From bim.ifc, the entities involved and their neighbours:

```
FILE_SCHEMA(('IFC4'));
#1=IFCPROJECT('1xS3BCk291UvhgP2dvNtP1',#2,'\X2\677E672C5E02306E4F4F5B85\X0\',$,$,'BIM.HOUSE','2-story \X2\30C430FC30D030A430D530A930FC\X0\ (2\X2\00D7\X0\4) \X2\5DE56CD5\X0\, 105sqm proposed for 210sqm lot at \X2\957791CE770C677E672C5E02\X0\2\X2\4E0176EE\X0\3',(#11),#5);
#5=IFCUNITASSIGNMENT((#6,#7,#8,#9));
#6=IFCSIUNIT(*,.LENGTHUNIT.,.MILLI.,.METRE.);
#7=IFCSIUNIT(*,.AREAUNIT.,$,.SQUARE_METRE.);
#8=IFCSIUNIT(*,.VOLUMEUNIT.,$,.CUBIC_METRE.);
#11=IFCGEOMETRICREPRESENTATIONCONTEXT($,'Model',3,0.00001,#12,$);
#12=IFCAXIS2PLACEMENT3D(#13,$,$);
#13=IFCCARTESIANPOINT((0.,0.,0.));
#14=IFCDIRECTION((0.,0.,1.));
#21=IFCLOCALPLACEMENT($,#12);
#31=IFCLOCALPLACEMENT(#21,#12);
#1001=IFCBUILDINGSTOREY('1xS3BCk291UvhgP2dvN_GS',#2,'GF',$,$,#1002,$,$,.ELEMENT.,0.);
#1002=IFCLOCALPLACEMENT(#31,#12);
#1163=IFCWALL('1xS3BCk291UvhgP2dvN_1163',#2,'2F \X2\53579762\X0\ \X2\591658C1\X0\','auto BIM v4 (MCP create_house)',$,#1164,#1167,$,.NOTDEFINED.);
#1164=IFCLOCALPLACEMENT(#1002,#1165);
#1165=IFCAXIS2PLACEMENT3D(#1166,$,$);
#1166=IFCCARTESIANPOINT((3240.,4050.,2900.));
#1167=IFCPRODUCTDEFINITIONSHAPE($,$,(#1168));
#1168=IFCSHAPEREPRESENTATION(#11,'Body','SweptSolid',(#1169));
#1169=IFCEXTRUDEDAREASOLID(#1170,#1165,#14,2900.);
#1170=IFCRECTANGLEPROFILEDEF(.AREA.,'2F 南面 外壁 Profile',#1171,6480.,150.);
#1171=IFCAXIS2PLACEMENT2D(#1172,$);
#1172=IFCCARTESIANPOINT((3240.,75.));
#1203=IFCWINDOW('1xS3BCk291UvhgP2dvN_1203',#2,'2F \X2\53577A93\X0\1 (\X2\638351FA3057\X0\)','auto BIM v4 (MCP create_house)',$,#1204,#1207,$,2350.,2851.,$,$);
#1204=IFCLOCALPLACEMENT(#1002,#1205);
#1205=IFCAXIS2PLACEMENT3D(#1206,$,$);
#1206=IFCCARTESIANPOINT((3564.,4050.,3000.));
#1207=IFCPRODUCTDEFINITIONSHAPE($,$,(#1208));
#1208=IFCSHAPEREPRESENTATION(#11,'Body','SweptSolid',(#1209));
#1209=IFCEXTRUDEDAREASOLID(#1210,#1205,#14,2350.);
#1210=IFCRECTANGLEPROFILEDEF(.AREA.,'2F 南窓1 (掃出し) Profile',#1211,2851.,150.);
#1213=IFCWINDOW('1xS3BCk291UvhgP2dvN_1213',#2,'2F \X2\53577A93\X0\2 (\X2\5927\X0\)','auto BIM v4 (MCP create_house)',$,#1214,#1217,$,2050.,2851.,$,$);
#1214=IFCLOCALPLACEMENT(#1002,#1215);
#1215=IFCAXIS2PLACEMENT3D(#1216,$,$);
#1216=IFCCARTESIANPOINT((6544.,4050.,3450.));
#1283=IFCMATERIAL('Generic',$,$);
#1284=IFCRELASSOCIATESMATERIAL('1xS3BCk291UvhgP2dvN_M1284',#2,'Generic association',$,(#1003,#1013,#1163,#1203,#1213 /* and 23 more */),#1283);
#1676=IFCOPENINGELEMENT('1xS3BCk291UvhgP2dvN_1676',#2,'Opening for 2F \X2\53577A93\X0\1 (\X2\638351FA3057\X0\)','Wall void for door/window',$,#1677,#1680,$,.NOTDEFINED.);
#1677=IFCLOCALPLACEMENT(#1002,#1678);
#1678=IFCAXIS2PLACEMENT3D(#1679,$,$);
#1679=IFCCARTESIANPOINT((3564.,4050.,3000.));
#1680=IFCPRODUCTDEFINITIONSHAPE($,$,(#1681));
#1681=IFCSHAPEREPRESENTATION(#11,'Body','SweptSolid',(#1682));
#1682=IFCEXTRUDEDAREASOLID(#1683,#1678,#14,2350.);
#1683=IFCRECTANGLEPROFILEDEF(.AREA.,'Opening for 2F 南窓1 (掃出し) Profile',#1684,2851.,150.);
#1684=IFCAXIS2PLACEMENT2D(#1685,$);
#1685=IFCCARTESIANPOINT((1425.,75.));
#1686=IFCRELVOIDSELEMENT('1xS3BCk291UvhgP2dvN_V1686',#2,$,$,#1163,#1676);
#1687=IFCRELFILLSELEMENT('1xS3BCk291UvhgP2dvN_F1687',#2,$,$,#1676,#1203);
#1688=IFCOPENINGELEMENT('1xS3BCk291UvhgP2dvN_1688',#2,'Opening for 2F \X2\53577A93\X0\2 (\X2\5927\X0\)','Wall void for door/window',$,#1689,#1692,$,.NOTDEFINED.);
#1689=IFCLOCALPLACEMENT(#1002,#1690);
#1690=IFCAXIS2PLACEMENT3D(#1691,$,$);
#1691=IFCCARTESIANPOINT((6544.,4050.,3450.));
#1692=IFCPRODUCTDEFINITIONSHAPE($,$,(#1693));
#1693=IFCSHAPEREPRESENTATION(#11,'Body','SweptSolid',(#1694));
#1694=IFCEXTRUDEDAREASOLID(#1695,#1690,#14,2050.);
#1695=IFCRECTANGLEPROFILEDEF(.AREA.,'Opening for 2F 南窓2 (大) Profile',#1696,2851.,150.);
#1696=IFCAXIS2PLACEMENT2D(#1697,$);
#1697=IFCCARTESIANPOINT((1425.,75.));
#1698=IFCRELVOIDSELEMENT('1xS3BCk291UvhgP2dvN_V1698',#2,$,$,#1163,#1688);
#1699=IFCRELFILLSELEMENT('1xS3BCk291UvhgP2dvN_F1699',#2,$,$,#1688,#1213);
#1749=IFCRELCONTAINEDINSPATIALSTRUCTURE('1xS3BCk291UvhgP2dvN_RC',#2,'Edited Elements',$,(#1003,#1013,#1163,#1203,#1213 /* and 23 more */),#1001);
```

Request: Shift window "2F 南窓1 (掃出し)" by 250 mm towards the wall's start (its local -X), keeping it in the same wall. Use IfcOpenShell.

```python
import ifcopenshell
import ifcopenshell.api.geometry
import ifcopenshell.util.placement
import ifcopenshell.util.unit

model = ifcopenshell.open("bim.ifc")
unit_scale = ifcopenshell.util.unit.calculate_unit_scale(model)

window = model.by_id(1203)
opening = window.FillsVoids[0].RelatingOpeningElement
wall = opening.VoidsElements[0].RelatingBuildingElement

wall_matrix = ifcopenshell.util.placement.get_local_placement(wall.ObjectPlacement)
shift = wall_matrix[:3, 0] * -0.25 / unit_scale
before = ifcopenshell.util.placement.get_local_placement(window.ObjectPlacement)[:3, 3].copy()

# The window is not placed relative to its opening, so move both.
for product in (opening, window):
    matrix = ifcopenshell.util.placement.get_local_placement(product.ObjectPlacement)
    matrix[:3, 3] += shift
    ifcopenshell.api.geometry.edit_object_placement(model, product=product, matrix=matrix, is_si=False)

after = ifcopenshell.util.placement.get_local_placement(window.ObjectPlacement)[:3, 3]
print("window moved by", (after - before).round(3) + 0.0)

model.write("bim_updated.ifc")
```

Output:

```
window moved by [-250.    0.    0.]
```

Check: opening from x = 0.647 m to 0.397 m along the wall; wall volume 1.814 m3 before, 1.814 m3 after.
